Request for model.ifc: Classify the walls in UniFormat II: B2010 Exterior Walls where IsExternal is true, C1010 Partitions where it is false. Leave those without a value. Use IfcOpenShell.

First a look at what the model holds.

```python
import ifcopenshell
import ifcopenshell.util.element

model = ifcopenshell.open("model.ifc")
print(model.schema)
print("classifications:", [c.Name for c in model.by_type("IfcClassification")])
values = [ifcopenshell.util.element.get_pset(e, "Pset_WallCommon", "IsExternal") for e in model.by_type("IfcWall")]
for value in (True, False, None):
    print("IsExternal", value, values.count(value))
```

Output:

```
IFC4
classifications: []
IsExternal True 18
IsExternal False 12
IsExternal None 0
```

```python
import ifcopenshell
import ifcopenshell.api.classification
import ifcopenshell.util.element

model = ifcopenshell.open("model.ifc")

system = ifcopenshell.api.classification.add_classification(model, classification="UniFormat II")

walls = model.by_type("IfcWall")
external = {e: ifcopenshell.util.element.get_pset(e, "Pset_WallCommon", "IsExternal") for e in walls}
for flag, code, name in ((True, "B2010", "Exterior Walls"), (False, "C1010", "Partitions")):
    products = [e for e in walls if external[e] is flag]
    ifcopenshell.api.classification.add_reference(
        model, products=products, classification=system, identification=code, name=name
    )
    print(code, len(products))

model.write("model_edited.ifc")
```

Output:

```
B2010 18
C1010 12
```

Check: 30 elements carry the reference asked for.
